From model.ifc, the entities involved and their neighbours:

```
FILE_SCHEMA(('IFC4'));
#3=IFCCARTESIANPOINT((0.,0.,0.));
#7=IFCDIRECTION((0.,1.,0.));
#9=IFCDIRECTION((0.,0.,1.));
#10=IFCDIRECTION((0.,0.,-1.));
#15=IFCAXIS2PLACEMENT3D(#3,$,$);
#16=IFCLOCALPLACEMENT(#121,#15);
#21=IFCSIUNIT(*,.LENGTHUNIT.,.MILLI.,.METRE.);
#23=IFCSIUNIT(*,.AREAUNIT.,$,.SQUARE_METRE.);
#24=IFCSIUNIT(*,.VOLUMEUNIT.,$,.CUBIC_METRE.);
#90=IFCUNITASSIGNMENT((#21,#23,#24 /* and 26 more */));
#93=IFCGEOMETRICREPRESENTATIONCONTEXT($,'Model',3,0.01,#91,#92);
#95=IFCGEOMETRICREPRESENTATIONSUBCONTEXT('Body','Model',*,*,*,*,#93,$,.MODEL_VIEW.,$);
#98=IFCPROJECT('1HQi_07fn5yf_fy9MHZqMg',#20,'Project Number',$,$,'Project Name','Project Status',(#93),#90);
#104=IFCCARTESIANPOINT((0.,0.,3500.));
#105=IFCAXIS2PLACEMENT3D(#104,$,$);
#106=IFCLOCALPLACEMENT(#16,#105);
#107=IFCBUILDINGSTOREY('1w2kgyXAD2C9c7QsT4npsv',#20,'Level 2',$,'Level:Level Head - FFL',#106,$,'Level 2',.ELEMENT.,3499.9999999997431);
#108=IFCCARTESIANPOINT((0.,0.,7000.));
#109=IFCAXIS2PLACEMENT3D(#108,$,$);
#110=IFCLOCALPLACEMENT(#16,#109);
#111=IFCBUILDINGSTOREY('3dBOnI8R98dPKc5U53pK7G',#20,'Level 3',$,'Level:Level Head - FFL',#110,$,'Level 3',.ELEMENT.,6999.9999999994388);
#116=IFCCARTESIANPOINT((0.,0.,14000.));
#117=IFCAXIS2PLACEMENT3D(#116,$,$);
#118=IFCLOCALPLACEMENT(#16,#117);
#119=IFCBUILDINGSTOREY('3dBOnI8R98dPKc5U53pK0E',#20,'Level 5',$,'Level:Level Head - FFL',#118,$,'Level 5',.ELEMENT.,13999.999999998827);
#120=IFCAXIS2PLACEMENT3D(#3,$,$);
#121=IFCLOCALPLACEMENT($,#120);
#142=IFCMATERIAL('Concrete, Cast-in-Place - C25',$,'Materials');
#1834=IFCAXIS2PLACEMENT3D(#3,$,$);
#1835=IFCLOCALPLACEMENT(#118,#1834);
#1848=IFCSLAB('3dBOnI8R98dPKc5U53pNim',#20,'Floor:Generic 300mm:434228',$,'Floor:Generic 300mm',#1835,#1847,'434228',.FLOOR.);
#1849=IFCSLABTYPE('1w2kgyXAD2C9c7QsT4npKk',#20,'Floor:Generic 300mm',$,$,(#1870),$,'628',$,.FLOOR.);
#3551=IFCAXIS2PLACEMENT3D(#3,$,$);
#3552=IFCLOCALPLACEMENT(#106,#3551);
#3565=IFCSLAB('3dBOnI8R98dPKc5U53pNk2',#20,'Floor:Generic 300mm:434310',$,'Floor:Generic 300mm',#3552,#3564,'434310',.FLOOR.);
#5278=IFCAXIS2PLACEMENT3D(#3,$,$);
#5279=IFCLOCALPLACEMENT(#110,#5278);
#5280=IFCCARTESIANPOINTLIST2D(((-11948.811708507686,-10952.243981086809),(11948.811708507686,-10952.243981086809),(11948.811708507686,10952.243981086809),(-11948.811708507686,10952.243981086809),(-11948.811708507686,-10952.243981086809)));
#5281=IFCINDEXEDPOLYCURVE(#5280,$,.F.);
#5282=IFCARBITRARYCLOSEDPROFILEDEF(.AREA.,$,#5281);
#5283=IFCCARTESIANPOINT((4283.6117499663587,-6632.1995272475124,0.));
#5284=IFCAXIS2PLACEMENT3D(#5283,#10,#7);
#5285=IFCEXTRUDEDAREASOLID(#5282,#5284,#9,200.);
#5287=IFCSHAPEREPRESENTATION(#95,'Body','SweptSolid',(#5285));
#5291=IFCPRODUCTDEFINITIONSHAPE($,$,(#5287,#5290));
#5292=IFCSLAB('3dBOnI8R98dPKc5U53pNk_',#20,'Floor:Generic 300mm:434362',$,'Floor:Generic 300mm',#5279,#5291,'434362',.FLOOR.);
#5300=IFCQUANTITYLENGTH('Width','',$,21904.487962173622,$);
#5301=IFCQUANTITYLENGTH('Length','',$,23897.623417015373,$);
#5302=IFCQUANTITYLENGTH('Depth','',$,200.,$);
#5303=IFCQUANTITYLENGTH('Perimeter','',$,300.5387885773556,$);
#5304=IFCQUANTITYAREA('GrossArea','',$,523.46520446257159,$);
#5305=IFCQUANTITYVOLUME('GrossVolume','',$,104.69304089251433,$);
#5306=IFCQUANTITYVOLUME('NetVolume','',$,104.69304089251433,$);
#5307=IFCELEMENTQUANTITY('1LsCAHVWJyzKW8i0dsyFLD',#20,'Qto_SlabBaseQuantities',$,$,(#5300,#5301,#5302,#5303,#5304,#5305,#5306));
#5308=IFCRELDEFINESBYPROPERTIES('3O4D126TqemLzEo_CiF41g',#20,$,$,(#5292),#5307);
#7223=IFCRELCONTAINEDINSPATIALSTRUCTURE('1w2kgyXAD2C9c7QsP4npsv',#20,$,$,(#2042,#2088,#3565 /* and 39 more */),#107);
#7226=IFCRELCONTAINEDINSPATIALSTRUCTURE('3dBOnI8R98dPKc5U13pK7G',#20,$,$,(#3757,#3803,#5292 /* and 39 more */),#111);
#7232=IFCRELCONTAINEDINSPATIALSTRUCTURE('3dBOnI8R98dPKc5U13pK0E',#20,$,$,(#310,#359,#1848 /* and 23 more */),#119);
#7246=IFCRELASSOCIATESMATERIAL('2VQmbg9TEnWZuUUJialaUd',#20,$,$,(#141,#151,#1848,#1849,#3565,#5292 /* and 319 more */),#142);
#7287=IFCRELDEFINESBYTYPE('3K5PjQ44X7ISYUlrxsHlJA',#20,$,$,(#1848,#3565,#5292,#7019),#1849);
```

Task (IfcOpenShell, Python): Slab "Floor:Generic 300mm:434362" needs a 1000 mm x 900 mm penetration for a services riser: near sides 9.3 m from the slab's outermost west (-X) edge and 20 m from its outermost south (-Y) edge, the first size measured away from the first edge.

```python
import numpy as np
import ifcopenshell
import ifcopenshell.api.feature
import ifcopenshell.api.geometry
import ifcopenshell.api.pset
import ifcopenshell.api.root
import ifcopenshell.geom
import ifcopenshell.util.element
import ifcopenshell.util.placement
import ifcopenshell.util.representation
import ifcopenshell.util.shape
import ifcopenshell.util.unit

model = ifcopenshell.open("model.ifc")
unit_scale = ifcopenshell.util.unit.calculate_unit_scale(model)
volume_scale = ifcopenshell.util.unit.calculate_unit_scale(model, "VOLUMEUNIT")
settings = ifcopenshell.geom.settings()


def volume(element):
    """Net volume in cubic metres, openings subtracted."""
    shape = ifcopenshell.geom.create_shape(settings, element)
    return ifcopenshell.util.shape.get_volume(shape.geometry)


slab = model.by_guid("3dBOnI8R98dPKc5U53pNk_")
before = volume(slab)

# Extent in the slab's own axes, in metres. The edges named are its -X and -Y sides.
slab_shape = ifcopenshell.geom.create_shape(settings, slab)
vertices = ifcopenshell.util.shape.get_vertices(slab_shape.geometry)
x_min, y_min, bottom = vertices.min(axis=0)
top = vertices[:, 2].max()

opening = ifcopenshell.api.root.create_entity(model, ifc_class="IfcOpeningElement", name="Services riser opening", predefined_type="OPENING")
context = ifcopenshell.util.representation.get_context(model, "Model", "Body", "MODEL_VIEW")
width, depth = 1, 0.9
outline = [(0.0, 0.0), (width, 0.0), (width, depth), (0.0, depth), (0.0, 0.0)]
# Overshoot both faces by 50 mm so the cut is clean.
shape = ifcopenshell.api.geometry.add_slab_representation(
    model, context=context, depth=top - bottom + 0.1, polyline=outline
)
ifcopenshell.api.geometry.assign_representation(model, product=opening, representation=shape)

matrix = ifcopenshell.util.placement.get_local_placement(slab.ObjectPlacement)
matrix[:, 3] = matrix @ np.append(np.array([x_min + 9.3, y_min + 20, bottom - 0.05]) / unit_scale, 1.0)
ifcopenshell.api.geometry.edit_object_placement(model, product=opening, matrix=matrix, is_si=False)
ifcopenshell.api.feature.add_feature(model, feature=opening, element=slab)

after = volume(slab)

# Update the slab's stored quantities.
qto = model.by_id(ifcopenshell.util.element.get_pset(slab, "Qto_SlabBaseQuantities", should_inherit=False)["id"])
ifcopenshell.api.pset.edit_qto(model, qto=qto, properties={"NetVolume": after / volume_scale})

print(f"slab volume {before:.3f} -> {after:.3f} m3")

model.write("model_rev.ifc")
```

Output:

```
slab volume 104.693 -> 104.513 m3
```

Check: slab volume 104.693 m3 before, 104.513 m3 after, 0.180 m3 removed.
